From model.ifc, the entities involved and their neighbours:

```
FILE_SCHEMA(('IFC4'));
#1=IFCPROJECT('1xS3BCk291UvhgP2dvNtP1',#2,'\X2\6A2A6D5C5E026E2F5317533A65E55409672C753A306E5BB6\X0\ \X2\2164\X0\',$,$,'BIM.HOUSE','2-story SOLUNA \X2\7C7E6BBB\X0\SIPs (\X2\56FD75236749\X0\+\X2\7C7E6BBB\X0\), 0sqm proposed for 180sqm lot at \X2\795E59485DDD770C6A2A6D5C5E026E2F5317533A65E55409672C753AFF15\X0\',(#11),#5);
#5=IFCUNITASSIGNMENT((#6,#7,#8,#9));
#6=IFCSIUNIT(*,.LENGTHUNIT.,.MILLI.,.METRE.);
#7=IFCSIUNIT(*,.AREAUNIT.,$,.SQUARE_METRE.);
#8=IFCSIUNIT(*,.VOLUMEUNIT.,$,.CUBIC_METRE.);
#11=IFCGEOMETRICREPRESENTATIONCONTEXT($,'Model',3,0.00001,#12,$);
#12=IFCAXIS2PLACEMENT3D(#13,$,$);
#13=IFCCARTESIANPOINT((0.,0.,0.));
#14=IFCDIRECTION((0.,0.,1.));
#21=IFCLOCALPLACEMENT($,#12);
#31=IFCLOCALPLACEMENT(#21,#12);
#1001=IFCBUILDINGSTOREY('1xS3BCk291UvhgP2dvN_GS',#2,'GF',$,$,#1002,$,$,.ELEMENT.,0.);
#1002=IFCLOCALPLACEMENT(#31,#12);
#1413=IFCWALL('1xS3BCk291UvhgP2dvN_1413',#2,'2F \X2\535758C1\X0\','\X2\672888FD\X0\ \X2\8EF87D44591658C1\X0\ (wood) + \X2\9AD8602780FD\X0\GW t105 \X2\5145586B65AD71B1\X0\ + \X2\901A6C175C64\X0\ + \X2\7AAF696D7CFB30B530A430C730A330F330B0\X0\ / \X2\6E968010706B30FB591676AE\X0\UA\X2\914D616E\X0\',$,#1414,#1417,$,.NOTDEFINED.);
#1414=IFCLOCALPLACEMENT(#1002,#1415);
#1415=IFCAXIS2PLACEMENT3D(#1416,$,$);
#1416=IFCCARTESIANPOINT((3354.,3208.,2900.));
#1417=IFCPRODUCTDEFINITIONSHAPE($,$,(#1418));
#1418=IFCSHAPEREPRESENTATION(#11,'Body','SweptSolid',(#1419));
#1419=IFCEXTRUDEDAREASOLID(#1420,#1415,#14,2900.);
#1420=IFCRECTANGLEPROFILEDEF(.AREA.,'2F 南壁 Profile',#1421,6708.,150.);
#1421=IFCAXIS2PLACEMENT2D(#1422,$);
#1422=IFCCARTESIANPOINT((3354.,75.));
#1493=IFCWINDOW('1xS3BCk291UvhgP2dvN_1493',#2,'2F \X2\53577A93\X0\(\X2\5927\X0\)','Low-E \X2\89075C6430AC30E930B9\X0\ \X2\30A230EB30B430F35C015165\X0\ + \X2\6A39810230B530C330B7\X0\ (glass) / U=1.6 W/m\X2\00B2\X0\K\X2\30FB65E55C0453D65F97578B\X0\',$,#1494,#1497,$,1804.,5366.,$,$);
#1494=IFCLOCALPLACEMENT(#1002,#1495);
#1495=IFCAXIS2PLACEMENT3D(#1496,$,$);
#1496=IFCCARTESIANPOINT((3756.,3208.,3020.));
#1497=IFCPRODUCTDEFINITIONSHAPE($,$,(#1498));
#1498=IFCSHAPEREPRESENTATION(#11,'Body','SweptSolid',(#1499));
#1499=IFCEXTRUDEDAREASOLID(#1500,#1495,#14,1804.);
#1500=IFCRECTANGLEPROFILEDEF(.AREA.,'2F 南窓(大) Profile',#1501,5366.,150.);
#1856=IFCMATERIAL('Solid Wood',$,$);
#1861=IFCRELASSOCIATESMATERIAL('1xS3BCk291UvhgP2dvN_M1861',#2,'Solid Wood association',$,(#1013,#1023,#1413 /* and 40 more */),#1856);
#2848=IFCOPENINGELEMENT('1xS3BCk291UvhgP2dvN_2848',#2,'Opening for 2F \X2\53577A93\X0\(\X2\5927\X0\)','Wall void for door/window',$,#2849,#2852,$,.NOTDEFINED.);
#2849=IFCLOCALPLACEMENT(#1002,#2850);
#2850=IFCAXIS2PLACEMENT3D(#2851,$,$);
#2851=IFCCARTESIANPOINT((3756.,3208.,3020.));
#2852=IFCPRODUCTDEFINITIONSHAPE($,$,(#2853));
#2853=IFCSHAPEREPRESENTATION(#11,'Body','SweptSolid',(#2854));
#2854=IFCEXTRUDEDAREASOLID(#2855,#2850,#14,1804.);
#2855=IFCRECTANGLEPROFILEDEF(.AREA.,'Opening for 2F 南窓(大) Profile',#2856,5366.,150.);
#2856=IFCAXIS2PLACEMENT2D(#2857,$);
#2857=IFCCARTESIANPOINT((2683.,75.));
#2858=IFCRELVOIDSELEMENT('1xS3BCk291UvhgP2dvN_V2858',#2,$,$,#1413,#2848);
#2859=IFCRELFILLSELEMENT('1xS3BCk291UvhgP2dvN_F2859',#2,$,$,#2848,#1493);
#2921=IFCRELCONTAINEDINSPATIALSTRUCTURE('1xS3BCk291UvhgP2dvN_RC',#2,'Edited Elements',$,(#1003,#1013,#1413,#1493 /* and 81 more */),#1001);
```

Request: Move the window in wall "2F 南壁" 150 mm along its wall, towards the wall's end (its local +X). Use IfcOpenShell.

```python
import ifcopenshell
import ifcopenshell.api.geometry
import ifcopenshell.util.placement
import ifcopenshell.util.unit

model = ifcopenshell.open("model.ifc")
unit_scale = ifcopenshell.util.unit.calculate_unit_scale(model)

window = model.by_guid("1xS3BCk291UvhgP2dvN_1493")
opening = window.FillsVoids[0].RelatingOpeningElement
wall = opening.VoidsElements[0].RelatingBuildingElement

wall_matrix = ifcopenshell.util.placement.get_local_placement(wall.ObjectPlacement)
shift = wall_matrix[:3, 0] * 0.15 / unit_scale
before = ifcopenshell.util.placement.get_local_placement(window.ObjectPlacement)[:3, 3].copy()

# The window is not placed relative to its opening, so move both.
for product in (opening, window):
    matrix = ifcopenshell.util.placement.get_local_placement(product.ObjectPlacement)
    matrix[:3, 3] += shift
    ifcopenshell.api.geometry.edit_object_placement(model, product=product, matrix=matrix, is_si=False)

after = ifcopenshell.util.placement.get_local_placement(window.ObjectPlacement)[:3, 3]
print("window moved by", (after - before).round(3) + 0.0)

model.write("model_edited.ifc")
```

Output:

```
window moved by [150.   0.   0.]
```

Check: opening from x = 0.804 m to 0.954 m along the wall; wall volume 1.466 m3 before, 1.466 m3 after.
